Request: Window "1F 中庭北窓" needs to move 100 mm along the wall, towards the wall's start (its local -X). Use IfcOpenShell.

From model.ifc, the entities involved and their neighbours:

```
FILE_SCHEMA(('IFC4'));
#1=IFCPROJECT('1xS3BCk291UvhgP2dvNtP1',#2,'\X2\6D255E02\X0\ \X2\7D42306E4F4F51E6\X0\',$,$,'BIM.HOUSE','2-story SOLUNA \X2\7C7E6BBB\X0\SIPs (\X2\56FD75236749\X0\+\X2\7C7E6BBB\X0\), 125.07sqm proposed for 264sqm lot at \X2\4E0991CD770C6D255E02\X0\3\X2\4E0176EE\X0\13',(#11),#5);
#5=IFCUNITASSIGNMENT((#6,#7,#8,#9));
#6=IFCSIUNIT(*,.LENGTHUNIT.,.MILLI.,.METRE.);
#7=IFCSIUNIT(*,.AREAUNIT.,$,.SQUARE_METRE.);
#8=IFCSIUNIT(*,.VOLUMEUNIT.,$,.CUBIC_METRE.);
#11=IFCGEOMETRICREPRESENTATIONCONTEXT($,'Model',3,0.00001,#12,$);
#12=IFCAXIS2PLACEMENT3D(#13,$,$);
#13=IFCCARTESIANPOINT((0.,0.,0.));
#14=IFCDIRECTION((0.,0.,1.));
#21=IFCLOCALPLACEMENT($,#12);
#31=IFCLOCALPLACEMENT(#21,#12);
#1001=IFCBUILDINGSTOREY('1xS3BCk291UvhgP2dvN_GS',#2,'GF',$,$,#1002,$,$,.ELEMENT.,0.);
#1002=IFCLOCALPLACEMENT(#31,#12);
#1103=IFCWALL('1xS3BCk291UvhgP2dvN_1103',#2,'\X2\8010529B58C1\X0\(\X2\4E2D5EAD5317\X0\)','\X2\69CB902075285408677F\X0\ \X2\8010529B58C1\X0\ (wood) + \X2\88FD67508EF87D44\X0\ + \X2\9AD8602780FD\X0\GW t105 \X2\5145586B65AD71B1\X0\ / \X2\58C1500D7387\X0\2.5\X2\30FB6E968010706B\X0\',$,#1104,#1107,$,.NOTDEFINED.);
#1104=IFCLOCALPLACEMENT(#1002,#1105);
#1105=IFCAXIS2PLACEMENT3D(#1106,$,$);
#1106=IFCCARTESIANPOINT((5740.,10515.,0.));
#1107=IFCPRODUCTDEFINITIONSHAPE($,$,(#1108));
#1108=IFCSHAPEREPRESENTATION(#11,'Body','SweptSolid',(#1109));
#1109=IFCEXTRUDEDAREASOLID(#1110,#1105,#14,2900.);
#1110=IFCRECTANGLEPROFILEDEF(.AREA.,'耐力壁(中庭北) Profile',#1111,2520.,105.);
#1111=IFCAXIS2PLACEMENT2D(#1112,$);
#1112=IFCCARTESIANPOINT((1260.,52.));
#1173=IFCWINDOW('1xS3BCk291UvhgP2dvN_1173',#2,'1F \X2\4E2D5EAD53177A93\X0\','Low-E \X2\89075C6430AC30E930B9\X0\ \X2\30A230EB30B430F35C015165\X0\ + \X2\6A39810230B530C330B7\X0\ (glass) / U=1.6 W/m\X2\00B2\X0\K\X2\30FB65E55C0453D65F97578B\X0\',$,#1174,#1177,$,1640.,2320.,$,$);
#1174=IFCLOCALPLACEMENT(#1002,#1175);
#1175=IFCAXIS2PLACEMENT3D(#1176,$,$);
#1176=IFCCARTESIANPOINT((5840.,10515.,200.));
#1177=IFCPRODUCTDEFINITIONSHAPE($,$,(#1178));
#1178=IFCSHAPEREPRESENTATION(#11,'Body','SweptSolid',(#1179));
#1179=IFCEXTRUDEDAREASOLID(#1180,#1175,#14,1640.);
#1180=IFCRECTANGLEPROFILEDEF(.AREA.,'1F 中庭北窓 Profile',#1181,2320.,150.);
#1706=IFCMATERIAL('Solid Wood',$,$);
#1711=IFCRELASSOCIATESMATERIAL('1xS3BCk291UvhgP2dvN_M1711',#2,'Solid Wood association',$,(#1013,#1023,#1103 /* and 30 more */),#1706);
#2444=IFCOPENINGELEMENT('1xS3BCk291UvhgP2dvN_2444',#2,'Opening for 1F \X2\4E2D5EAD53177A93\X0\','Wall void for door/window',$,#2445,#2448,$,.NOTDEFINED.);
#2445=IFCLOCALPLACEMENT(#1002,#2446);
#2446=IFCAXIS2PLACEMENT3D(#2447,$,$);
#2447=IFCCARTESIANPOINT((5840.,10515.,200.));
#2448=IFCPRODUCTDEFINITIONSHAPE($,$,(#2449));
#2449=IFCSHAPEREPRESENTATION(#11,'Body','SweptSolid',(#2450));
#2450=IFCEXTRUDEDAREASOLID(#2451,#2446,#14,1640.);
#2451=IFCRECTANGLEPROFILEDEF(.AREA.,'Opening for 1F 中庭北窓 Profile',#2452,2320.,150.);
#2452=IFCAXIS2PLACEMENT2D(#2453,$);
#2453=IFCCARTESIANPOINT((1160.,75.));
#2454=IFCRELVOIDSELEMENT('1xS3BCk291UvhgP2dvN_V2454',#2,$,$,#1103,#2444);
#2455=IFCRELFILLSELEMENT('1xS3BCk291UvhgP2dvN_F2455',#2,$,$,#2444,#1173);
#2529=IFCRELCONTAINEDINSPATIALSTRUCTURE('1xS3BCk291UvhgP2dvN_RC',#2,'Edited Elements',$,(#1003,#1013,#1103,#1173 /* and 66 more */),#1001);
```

```python
import ifcopenshell
import ifcopenshell.api.geometry
import ifcopenshell.util.placement
import ifcopenshell.util.unit

model = ifcopenshell.open("model.ifc")
unit_scale = ifcopenshell.util.unit.calculate_unit_scale(model)

window = model.by_guid("1xS3BCk291UvhgP2dvN_1173")
opening = window.FillsVoids[0].RelatingOpeningElement
wall = opening.VoidsElements[0].RelatingBuildingElement

wall_matrix = ifcopenshell.util.placement.get_local_placement(wall.ObjectPlacement)
shift = wall_matrix[:3, 0] * -0.1 / unit_scale
before = ifcopenshell.util.placement.get_local_placement(window.ObjectPlacement)[:3, 3].copy()

# The window is not placed relative to its opening, so move both.
for product in (opening, window):
    matrix = ifcopenshell.util.placement.get_local_placement(product.ObjectPlacement)
    matrix[:3, 3] += shift
    ifcopenshell.api.geometry.edit_object_placement(model, product=product, matrix=matrix, is_si=False)

after = ifcopenshell.util.placement.get_local_placement(window.ObjectPlacement)[:3, 3]
print("window moved by", (after - before).round(3) + 0.0)

model.write("model_edited.ifc")
```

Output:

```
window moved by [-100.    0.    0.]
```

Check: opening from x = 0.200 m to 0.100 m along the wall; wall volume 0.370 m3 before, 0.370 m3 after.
